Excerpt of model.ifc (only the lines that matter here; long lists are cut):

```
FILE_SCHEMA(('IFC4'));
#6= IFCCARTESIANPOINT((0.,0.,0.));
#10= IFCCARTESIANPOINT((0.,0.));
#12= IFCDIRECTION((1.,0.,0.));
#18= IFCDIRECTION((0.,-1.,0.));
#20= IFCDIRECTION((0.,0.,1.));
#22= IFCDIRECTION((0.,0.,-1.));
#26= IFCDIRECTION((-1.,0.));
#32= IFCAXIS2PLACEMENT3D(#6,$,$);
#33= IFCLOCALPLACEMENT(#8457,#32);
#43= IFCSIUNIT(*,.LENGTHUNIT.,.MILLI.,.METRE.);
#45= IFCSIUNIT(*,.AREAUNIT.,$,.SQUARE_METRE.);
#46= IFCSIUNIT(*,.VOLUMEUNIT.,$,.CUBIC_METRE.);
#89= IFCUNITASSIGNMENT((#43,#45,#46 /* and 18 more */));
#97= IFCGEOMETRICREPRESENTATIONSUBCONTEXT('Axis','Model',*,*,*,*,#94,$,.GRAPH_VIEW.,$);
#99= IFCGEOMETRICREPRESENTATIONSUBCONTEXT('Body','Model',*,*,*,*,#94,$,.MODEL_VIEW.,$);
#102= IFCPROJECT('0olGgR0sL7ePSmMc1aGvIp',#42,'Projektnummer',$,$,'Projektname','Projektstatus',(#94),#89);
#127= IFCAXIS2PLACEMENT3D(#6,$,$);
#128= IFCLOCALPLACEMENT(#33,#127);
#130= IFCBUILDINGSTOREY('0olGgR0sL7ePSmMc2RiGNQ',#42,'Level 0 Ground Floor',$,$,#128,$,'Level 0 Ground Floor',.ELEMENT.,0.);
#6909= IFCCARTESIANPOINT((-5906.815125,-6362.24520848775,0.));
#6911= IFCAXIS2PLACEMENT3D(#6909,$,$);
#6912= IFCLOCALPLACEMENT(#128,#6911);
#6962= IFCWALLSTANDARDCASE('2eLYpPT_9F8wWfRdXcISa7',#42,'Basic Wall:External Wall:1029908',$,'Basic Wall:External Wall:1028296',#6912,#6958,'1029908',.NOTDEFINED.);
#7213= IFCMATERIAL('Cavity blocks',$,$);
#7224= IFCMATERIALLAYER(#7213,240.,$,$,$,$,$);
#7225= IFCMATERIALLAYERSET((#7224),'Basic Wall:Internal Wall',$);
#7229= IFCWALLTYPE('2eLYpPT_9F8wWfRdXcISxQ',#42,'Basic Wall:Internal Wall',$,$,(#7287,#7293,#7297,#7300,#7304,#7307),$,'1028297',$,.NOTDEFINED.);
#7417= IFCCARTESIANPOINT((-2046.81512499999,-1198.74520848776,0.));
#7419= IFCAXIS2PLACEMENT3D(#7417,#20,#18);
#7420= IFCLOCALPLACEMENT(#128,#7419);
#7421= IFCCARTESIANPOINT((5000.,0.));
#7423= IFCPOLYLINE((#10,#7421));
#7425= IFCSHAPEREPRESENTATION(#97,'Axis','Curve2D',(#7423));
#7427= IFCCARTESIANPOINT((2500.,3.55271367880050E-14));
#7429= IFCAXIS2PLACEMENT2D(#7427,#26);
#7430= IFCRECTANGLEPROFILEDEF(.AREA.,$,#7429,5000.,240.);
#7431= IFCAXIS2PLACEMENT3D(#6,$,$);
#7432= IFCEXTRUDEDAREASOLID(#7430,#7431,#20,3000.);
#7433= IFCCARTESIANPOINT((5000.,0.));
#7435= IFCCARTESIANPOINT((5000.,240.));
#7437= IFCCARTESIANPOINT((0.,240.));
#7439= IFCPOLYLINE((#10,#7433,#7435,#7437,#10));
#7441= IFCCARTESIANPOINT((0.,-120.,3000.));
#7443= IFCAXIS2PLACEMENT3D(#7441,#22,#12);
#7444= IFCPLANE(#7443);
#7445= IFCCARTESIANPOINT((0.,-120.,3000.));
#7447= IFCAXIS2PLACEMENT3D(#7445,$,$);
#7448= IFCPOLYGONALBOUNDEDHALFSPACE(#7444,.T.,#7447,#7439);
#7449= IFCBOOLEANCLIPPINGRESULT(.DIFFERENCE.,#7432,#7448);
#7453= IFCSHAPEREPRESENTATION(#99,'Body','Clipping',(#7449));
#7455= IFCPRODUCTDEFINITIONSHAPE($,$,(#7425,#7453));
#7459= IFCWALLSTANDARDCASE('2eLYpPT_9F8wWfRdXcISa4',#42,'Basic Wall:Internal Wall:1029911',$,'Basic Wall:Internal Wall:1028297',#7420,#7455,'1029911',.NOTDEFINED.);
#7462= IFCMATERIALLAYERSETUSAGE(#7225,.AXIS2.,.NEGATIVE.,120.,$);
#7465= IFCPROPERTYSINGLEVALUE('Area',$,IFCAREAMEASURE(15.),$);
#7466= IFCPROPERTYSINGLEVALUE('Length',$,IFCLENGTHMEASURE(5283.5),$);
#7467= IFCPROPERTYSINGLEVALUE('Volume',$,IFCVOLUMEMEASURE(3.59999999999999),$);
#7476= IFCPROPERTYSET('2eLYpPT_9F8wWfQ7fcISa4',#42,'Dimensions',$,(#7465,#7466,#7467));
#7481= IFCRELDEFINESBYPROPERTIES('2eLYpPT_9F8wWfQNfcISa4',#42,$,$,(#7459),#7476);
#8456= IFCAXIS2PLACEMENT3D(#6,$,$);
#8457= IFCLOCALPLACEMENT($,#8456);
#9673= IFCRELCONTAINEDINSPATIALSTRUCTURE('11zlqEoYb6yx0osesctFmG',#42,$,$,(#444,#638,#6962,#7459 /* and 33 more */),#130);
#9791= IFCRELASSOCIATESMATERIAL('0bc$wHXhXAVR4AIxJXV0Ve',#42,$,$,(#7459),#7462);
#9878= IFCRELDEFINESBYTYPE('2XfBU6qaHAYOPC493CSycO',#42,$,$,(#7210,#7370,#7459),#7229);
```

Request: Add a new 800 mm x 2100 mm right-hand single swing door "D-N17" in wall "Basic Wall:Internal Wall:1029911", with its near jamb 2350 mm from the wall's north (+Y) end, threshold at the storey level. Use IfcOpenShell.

```python
import numpy as np
import ifcopenshell
import ifcopenshell.api.feature
import ifcopenshell.api.geometry
import ifcopenshell.api.pset
import ifcopenshell.api.root
import ifcopenshell.api.spatial
import ifcopenshell.geom
import ifcopenshell.util.element
import ifcopenshell.util.placement
import ifcopenshell.util.representation
import ifcopenshell.util.shape
import ifcopenshell.util.unit

model = ifcopenshell.open("model.ifc")
unit_scale = ifcopenshell.util.unit.calculate_unit_scale(model)
area_scale = ifcopenshell.util.unit.calculate_unit_scale(model, "AREAUNIT")
volume_scale = ifcopenshell.util.unit.calculate_unit_scale(model, "VOLUMEUNIT")
settings = ifcopenshell.geom.settings()


def volume(element):
    """Net volume in cubic metres, openings subtracted."""
    shape = ifcopenshell.geom.create_shape(settings, element)
    return ifcopenshell.util.shape.get_volume(shape.geometry)


wall = model.by_id(7459)
storey = ifcopenshell.util.element.get_container(wall, ifc_class="IfcBuildingStorey")
context = ifcopenshell.util.representation.get_context(model, "Model", "Body", "MODEL_VIEW")
before = volume(wall)

width, height, from_end, sill = 0.8, 2.1, 2.35, 0.0  # metres

# The wall runs along its own X axis, and the end named is its -X end.
wall_shape = ifcopenshell.geom.create_shape(settings, wall)
x, y, z = ifcopenshell.util.shape.get_vertices(wall_shape.geometry).T
start = x.min() + from_end
face, thickness = float(y.min()), float(y.max() - y.min())
wall_matrix = ifcopenshell.util.placement.get_local_placement(wall.ObjectPlacement)
level = ifcopenshell.util.placement.get_local_placement(storey.ObjectPlacement)[2, 3]


def in_wall(x, y):
    """Placement at x, y metres in the wall's axes, at sill height."""
    matrix = wall_matrix.copy()
    matrix[:, 3] = wall_matrix @ np.array([x / unit_scale, y / unit_scale, 0.0, 1.0])
    matrix[2, 3] = level + sill / unit_scale
    return matrix


# Opening: a box that overshoots both wall faces by 50 mm.
opening = ifcopenshell.api.root.create_entity(model, ifc_class="IfcOpeningElement", predefined_type="OPENING")
box = ifcopenshell.api.geometry.add_wall_representation(
    model, context=context, length=width, height=height, thickness=thickness + 0.1
)
ifcopenshell.api.geometry.assign_representation(model, product=opening, representation=box)
ifcopenshell.api.geometry.edit_object_placement(model, product=opening, matrix=in_wall(start, face - 0.05), is_si=False)
ifcopenshell.api.feature.add_feature(model, feature=opening, element=wall)

door = ifcopenshell.api.root.create_entity(model, ifc_class="IfcDoor", name="D-N17", predefined_type="DOOR")
door.OverallWidth, door.OverallHeight = width / unit_scale, height / unit_scale
door.OperationType = "SINGLE_SWING_RIGHT"
body = ifcopenshell.api.geometry.add_door_representation(
    model,
    context=context,
    overall_width=door.OverallWidth,
    overall_height=door.OverallHeight,
    operation_type="SINGLE_SWING_RIGHT",
    lining_properties={"LiningDepth": thickness / unit_scale, "ThresholdDepth": thickness / unit_scale},
)
ifcopenshell.api.geometry.assign_representation(model, product=door, representation=body)
ifcopenshell.api.spatial.assign_container(model, products=[door], relating_structure=storey)
ifcopenshell.api.feature.add_filling(model, opening=opening, element=door)

# The lining spans the wall, so the door starts at the wall face.
ifcopenshell.api.geometry.edit_object_placement(model, product=door, matrix=in_wall(start, face), is_si=False)

after = volume(wall)

# Update the wall's stored quantities.
pset = model.by_id(ifcopenshell.util.element.get_pset(wall, "Dimensions", should_inherit=False)["id"])
ifcopenshell.api.pset.edit_pset(model, pset=pset, properties={
    "Area": model.create_entity("IfcAreaMeasure", after / thickness / area_scale),
    "Volume": model.create_entity("IfcVolumeMeasure", after / volume_scale),
})

print(f"wall volume {before:.3f} -> {after:.3f} m3")

model.write("model_v2.ifc")
```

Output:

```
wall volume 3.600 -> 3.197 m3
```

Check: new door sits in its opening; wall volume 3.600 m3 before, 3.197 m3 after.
